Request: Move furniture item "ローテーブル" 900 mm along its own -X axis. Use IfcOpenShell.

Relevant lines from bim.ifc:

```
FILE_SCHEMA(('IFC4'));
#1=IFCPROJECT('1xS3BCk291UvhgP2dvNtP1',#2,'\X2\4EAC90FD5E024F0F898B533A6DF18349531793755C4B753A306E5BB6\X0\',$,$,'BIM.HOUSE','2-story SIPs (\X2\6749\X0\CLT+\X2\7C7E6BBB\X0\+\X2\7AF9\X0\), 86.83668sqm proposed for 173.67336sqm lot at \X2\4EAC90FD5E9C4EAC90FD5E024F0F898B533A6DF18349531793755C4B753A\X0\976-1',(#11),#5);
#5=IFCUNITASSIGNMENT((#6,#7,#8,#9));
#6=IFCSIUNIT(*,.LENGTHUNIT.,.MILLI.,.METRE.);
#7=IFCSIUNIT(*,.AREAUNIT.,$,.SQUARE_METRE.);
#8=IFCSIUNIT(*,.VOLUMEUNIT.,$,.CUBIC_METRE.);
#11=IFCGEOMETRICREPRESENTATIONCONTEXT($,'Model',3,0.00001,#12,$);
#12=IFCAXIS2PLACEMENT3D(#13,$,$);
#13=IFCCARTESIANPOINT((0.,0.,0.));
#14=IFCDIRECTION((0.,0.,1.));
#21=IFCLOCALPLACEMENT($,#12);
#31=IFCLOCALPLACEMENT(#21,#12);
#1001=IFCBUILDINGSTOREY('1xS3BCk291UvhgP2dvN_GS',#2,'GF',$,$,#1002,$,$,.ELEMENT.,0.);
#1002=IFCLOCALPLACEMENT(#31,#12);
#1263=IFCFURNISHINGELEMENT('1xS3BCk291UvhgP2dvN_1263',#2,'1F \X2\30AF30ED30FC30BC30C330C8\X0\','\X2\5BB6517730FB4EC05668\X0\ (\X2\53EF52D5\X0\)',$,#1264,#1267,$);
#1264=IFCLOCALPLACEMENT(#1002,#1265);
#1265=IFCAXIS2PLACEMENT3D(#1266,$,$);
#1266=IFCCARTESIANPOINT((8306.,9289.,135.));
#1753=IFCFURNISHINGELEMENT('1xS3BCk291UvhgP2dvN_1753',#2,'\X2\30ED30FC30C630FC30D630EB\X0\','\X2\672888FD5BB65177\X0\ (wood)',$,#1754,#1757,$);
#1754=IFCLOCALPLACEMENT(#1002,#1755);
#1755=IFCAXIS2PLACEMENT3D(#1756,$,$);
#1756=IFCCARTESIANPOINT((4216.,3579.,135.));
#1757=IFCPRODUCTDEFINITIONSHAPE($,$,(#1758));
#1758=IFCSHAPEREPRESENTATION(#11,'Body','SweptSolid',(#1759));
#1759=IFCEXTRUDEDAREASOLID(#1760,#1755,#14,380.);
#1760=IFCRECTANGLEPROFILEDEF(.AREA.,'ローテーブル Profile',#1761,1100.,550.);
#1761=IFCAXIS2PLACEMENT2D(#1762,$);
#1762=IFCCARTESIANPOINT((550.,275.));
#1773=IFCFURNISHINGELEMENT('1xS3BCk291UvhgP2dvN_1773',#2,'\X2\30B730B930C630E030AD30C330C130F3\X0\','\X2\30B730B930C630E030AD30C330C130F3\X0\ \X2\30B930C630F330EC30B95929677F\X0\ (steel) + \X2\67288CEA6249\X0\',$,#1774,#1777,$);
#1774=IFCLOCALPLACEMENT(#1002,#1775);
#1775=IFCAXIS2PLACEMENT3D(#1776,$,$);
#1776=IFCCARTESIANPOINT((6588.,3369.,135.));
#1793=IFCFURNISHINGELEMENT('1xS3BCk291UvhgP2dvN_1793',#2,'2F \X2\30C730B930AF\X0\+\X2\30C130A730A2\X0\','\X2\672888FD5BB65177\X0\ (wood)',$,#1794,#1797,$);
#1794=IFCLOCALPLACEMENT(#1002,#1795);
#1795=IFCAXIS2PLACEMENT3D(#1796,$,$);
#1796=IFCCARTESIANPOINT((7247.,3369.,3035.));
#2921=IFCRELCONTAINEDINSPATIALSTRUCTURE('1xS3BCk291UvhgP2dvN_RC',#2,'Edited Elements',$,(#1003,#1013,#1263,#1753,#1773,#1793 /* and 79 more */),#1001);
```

```python
import ifcopenshell
import ifcopenshell.api.geometry
import ifcopenshell.util.placement
import ifcopenshell.util.unit

model = ifcopenshell.open("bim.ifc")
unit_scale = ifcopenshell.util.unit.calculate_unit_scale(model)

item = model.by_guid("1xS3BCk291UvhgP2dvN_1753")
matrix = ifcopenshell.util.placement.get_local_placement(item.ObjectPlacement)
matrix[:3, 3] -= matrix[:3, 0] * 0.9 / unit_scale
ifcopenshell.api.geometry.edit_object_placement(model, product=item, matrix=matrix, is_si=False)

print(ifcopenshell.util.placement.get_local_placement(item.ObjectPlacement).round(3) + 0.0)

model.write("bim_updated.ifc")
```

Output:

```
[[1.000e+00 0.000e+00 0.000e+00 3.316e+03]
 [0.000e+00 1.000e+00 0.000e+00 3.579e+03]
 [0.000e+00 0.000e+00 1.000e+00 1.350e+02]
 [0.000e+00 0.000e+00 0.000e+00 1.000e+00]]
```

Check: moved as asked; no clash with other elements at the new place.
